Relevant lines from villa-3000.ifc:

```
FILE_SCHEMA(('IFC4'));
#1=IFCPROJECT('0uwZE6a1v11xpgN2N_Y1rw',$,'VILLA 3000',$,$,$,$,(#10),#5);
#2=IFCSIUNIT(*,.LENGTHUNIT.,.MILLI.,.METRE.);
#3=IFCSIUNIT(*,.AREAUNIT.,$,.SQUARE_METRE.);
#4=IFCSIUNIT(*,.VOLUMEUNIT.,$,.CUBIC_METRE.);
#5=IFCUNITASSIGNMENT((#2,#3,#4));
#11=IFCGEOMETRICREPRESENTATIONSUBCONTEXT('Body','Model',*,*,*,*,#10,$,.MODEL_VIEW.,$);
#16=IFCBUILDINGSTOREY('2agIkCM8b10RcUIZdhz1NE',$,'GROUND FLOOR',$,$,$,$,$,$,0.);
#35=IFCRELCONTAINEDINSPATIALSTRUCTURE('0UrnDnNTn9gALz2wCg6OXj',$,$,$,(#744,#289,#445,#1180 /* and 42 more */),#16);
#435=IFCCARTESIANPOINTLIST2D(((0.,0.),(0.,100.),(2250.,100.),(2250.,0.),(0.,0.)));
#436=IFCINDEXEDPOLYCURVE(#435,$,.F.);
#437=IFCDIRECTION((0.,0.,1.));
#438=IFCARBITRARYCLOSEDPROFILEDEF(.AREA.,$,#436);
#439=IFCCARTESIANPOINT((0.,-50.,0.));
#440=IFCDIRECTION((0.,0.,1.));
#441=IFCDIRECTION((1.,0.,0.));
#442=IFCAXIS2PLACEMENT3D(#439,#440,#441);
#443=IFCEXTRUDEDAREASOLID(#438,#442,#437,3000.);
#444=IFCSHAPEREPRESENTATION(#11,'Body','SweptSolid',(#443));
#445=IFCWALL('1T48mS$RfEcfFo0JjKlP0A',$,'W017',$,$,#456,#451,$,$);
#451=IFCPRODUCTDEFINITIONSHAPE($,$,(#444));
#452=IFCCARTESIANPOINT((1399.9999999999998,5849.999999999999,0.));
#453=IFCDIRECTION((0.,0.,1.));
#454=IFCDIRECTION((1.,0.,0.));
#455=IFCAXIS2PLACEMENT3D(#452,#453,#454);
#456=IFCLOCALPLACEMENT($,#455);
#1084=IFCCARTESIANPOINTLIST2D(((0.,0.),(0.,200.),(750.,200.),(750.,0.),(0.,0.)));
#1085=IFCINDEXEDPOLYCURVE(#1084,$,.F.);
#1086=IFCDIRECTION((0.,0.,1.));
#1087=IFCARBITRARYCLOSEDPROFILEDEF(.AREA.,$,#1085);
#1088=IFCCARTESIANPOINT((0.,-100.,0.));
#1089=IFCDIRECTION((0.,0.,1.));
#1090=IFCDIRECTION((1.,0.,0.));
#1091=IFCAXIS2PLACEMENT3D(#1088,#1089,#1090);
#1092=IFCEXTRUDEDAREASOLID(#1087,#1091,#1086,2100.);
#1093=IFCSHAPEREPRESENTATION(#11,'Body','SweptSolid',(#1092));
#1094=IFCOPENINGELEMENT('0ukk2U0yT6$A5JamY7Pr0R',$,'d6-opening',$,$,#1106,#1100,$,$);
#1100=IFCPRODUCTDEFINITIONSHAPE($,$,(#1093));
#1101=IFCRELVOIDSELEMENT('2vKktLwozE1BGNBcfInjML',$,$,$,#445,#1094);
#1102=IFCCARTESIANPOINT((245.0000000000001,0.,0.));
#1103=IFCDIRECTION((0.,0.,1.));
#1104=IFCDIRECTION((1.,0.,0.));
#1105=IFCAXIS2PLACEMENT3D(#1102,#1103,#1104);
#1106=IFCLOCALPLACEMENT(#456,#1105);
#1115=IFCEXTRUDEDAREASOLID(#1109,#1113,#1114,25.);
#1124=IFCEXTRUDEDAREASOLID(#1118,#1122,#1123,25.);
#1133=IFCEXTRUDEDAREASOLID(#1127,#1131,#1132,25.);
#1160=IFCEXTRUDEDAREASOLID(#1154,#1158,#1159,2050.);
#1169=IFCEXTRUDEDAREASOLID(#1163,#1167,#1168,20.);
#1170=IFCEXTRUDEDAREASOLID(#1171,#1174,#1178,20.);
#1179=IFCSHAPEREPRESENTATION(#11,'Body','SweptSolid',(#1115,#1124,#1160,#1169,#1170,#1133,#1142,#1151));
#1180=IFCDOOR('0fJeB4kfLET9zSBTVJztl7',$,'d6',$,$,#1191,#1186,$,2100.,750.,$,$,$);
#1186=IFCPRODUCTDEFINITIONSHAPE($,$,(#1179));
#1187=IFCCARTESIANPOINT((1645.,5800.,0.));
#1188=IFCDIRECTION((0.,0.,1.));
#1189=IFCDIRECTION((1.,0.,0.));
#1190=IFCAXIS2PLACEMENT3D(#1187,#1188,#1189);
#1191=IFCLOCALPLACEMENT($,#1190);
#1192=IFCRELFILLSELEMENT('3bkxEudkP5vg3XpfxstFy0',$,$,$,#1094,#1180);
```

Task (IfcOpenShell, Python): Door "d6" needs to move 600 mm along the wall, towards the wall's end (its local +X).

```python
import ifcopenshell
import ifcopenshell.api.geometry
import ifcopenshell.util.placement

model = ifcopenshell.open("villa-3000.ifc")

door = model.by_id(1180)
opening = door.FillsVoids[0].RelatingOpeningElement
wall = opening.VoidsElements[0].RelatingBuildingElement

wall_matrix = ifcopenshell.util.placement.get_local_placement(wall.ObjectPlacement)
shift = wall_matrix[:3, 0] * 600.0
before = ifcopenshell.util.placement.get_local_placement(door.ObjectPlacement)[:3, 3].copy()

# The door is not placed relative to its opening, so move both.
for product in (opening, door):
    matrix = ifcopenshell.util.placement.get_local_placement(product.ObjectPlacement)
    matrix[:3, 3] += shift
    ifcopenshell.api.geometry.edit_object_placement(model, product=product, matrix=matrix, is_si=False)

after = ifcopenshell.util.placement.get_local_placement(door.ObjectPlacement)[:3, 3]
print("door moved by", (after - before).round(3) + 0.0)

model.write("villa-3000_updated.ifc")
```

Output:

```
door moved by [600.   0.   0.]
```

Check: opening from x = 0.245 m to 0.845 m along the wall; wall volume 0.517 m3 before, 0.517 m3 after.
